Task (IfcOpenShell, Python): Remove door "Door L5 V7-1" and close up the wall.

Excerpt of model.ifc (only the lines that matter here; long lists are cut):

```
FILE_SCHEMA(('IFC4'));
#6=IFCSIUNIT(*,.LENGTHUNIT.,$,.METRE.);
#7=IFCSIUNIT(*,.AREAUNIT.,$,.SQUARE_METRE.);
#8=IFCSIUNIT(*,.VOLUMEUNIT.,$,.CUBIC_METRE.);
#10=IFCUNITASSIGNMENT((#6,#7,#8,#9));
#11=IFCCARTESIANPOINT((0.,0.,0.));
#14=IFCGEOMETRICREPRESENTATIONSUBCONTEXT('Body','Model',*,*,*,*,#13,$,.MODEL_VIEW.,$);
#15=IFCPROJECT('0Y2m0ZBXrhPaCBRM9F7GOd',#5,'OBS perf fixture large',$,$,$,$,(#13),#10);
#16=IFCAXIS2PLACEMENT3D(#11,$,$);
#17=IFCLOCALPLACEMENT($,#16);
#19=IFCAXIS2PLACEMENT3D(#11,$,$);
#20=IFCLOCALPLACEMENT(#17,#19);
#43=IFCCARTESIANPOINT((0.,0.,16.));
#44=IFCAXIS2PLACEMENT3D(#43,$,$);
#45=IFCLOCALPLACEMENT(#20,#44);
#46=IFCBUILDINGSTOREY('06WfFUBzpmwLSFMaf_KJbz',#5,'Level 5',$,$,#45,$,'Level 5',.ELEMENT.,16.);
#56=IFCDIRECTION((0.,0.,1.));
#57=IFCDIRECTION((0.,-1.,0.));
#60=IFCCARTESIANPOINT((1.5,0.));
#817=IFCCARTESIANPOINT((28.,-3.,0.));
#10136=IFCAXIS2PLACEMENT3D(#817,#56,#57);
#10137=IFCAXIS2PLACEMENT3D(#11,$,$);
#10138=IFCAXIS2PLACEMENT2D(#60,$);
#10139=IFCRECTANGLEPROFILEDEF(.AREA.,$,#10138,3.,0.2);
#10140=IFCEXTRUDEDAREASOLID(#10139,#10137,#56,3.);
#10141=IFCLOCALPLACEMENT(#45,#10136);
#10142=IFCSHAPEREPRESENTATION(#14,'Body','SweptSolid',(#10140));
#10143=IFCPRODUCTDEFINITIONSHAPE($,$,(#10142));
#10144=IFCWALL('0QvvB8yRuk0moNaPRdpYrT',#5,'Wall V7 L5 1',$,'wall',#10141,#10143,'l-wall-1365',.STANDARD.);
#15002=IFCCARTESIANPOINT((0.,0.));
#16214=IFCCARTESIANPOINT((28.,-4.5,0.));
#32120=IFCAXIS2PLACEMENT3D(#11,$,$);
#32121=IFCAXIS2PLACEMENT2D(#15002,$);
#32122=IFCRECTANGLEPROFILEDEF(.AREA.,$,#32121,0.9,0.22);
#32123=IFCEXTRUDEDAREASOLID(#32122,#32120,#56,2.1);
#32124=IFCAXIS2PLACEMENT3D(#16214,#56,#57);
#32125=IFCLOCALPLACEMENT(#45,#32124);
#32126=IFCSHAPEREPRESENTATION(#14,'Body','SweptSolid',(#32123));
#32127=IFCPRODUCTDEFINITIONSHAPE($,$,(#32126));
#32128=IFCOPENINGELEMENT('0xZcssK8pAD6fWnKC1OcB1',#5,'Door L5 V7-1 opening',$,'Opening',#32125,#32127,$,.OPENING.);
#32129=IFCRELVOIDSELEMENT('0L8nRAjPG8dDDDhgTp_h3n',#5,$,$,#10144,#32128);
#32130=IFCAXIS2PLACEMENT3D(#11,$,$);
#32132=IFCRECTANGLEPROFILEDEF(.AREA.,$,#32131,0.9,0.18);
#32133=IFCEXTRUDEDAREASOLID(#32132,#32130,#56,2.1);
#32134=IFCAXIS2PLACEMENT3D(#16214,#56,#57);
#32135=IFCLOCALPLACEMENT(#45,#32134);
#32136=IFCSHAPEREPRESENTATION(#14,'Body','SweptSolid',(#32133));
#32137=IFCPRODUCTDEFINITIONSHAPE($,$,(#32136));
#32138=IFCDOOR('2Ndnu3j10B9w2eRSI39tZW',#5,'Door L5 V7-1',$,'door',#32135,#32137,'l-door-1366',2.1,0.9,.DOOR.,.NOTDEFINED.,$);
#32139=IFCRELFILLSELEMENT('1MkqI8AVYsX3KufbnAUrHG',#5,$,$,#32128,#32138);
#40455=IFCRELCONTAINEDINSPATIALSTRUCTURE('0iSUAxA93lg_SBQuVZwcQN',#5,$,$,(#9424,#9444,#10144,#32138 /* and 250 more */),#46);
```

```python
import ifcopenshell
import ifcopenshell.api.feature
import ifcopenshell.api.root
import ifcopenshell.geom
import ifcopenshell.util.shape

model = ifcopenshell.open("model.ifc")
settings = ifcopenshell.geom.settings()


def volume(element):
    """Net volume in cubic metres, openings subtracted."""
    shape = ifcopenshell.geom.create_shape(settings, element)
    return ifcopenshell.util.shape.get_volume(shape.geometry)


door = model.by_id(32138)
opening = door.FillsVoids[0].RelatingOpeningElement
wall = opening.VoidsElements[0].RelatingBuildingElement
before = volume(wall)

ifcopenshell.api.root.remove_product(model, product=door)
ifcopenshell.api.feature.remove_feature(model, feature=opening)

after = volume(wall)

print(f"wall volume {before:.3f} -> {after:.3f} m3")

model.write("model_v2.ifc")
```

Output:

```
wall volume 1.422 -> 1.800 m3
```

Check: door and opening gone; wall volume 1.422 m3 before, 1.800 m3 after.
